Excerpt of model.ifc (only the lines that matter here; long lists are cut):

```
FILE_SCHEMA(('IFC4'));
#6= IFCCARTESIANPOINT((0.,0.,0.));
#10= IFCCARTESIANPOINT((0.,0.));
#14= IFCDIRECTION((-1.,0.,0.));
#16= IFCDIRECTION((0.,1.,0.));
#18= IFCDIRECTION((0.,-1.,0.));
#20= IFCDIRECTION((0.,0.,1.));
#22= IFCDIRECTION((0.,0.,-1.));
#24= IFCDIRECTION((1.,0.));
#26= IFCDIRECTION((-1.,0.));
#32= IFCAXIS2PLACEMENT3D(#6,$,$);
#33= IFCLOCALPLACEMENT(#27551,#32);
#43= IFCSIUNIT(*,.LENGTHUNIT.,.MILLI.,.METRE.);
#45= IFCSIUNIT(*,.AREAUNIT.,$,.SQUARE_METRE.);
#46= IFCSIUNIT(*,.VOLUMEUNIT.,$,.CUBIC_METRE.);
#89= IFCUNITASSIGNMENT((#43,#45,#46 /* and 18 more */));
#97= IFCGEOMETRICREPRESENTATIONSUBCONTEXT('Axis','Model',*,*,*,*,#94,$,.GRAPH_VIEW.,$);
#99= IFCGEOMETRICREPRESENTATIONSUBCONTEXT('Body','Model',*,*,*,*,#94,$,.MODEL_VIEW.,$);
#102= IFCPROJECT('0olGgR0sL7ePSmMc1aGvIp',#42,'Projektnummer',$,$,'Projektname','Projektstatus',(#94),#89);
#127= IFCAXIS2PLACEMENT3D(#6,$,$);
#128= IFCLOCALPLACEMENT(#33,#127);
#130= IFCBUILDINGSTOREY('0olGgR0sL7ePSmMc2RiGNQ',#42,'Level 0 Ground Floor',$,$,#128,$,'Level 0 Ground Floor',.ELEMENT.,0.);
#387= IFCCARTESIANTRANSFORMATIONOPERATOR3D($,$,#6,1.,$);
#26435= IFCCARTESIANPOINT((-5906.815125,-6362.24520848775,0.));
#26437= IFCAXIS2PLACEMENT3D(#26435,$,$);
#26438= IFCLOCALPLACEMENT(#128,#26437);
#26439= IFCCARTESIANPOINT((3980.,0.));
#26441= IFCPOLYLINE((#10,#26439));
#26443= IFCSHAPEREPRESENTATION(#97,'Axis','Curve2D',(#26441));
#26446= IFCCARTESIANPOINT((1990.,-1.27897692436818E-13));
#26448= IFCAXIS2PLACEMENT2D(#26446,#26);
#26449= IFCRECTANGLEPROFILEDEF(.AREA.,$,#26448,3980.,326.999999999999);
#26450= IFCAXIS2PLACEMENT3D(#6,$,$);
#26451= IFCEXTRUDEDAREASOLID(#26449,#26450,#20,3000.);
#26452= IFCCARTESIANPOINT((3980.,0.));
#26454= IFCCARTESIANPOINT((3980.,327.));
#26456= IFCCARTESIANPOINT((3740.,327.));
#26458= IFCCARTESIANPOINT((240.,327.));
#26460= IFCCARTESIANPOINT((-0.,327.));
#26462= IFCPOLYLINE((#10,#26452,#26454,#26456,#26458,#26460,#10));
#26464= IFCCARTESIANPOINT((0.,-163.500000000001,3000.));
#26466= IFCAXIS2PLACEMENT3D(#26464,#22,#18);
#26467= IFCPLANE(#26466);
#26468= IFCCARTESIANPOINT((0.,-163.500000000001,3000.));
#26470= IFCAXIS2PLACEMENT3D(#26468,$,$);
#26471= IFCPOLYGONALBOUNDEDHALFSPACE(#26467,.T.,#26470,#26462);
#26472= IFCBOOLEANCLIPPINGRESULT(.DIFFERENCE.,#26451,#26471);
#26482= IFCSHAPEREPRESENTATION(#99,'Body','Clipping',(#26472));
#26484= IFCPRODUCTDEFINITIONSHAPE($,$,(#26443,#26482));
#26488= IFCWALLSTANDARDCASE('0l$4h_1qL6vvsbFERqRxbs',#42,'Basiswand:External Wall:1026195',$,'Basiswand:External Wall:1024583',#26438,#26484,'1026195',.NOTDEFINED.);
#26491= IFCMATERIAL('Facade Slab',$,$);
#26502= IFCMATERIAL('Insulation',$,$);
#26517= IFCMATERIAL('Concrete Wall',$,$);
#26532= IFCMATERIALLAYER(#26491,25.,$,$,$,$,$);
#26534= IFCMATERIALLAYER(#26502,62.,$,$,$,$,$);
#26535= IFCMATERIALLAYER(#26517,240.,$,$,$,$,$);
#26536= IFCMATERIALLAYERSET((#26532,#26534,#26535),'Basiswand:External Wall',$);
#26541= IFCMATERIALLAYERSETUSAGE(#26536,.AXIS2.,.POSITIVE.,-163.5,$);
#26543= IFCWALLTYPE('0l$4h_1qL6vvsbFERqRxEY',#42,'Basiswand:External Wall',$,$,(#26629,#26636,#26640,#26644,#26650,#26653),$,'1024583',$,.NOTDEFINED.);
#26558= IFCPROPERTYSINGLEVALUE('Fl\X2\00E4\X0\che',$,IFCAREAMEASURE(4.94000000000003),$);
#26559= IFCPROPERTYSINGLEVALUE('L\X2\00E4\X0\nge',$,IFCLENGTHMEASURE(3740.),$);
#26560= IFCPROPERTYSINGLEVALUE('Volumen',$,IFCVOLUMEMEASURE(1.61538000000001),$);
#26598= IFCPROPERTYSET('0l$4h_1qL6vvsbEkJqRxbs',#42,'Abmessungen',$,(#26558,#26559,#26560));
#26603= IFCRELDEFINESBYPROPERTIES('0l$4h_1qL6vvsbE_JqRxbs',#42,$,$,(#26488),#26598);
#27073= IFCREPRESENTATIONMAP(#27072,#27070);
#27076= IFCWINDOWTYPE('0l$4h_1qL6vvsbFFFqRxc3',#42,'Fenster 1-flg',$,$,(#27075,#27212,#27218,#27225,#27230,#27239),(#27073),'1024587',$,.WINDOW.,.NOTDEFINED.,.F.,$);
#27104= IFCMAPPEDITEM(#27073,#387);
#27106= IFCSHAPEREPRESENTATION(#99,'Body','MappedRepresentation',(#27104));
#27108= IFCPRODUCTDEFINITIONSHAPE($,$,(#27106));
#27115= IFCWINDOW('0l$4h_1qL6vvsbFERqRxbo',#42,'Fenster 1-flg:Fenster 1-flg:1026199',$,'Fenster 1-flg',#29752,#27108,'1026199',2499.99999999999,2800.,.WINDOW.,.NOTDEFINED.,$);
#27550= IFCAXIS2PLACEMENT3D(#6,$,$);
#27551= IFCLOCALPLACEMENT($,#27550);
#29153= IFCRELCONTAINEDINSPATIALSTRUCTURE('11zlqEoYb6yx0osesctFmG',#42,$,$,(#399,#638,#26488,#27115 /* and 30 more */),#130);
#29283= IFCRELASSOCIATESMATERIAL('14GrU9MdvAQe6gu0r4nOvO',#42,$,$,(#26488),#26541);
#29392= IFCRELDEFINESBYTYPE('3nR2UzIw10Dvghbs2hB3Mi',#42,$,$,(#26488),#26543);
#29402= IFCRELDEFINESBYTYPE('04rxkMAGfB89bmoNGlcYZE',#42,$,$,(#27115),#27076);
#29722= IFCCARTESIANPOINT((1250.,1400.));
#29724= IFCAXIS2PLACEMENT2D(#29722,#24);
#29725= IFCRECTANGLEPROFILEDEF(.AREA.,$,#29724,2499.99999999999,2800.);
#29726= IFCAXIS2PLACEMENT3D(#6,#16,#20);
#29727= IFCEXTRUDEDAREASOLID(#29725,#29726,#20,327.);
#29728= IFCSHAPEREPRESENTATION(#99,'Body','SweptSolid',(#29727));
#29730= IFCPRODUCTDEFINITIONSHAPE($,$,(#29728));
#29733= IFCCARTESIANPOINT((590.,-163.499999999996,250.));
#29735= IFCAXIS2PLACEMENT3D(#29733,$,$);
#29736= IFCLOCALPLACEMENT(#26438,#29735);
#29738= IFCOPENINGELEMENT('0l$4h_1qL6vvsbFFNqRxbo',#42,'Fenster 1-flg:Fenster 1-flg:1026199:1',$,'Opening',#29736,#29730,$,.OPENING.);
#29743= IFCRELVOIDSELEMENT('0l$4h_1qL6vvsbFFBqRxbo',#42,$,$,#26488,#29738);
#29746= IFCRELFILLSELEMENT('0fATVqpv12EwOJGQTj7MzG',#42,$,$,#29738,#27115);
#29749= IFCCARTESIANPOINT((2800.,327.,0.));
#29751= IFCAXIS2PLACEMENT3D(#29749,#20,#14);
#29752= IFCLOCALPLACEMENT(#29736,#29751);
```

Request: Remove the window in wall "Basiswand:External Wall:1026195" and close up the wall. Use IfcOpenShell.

```python
import ifcopenshell
import ifcopenshell.api.feature
import ifcopenshell.api.pset
import ifcopenshell.api.root
import ifcopenshell.geom
import ifcopenshell.util.element
import ifcopenshell.util.shape
import ifcopenshell.util.unit

model = ifcopenshell.open("model.ifc")
area_scale = ifcopenshell.util.unit.calculate_unit_scale(model, "AREAUNIT")
volume_scale = ifcopenshell.util.unit.calculate_unit_scale(model, "VOLUMEUNIT")
settings = ifcopenshell.geom.settings()


def volume(element):
    """Net volume in cubic metres, openings subtracted."""
    shape = ifcopenshell.geom.create_shape(settings, element)
    return ifcopenshell.util.shape.get_volume(shape.geometry)


window = model.by_guid("0l$4h_1qL6vvsbFERqRxbo")
opening = window.FillsVoids[0].RelatingOpeningElement
wall = opening.VoidsElements[0].RelatingBuildingElement
before = volume(wall)

ifcopenshell.api.root.remove_product(model, product=window)
ifcopenshell.api.feature.remove_feature(model, feature=opening)

after = volume(wall)
thickness = 0.327  # wall thickness in metres

# Update the wall's stored quantities.
pset = model.by_id(ifcopenshell.util.element.get_pset(wall, "Abmessungen", should_inherit=False)["id"])
ifcopenshell.api.pset.edit_pset(model, pset=pset, properties={
    "Fläche": model.create_entity("IfcAreaMeasure", after / thickness / area_scale),
    "Volumen": model.create_entity("IfcVolumeMeasure", after / volume_scale),
})

print(f"wall volume {before:.3f} -> {after:.3f} m3")

model.write("model_updated.ifc")
```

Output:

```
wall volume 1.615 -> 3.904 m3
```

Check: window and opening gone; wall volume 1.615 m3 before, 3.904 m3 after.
